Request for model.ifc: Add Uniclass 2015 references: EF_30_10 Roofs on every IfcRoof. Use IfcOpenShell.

First a look at what the model holds.

```python
import ifcopenshell

model = ifcopenshell.open("model.ifc")
print(model.schema)
print("classifications:", [c.Name for c in model.by_type("IfcClassification")])
for ifc_class in ("IfcDoor", "IfcRoof", "IfcStair", "IfcWall", "IfcWindow"):
    print(ifc_class, len(model.by_type(ifc_class)))
```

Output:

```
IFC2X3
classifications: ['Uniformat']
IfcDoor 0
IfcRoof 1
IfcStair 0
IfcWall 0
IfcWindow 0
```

```python
import ifcopenshell
import ifcopenshell.api.classification

model = ifcopenshell.open("model.ifc")

# IFC2X3 requires Source and Edition and has no link from the project to the system.
system = model.create_entity("IfcClassification", Source="NBS", Edition="2015", Name="Uniclass 2015")

codes = {
    "IfcRoof": ("EF_30_10", "Roofs"),
}
for ifc_class, (code, name) in codes.items():
    products = model.by_type(ifc_class)
    ifcopenshell.api.classification.add_reference(
        model, products=products, classification=system, identification=code, name=name
    )
    print(code, len(products))

model.write("model_updated.ifc")
```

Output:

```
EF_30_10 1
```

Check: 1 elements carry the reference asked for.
